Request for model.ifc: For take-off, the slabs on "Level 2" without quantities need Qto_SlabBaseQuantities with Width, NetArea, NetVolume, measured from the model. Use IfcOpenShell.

First a look at what the model holds.

```python
import ifcopenshell
import ifcopenshell.util.element
import ifcopenshell.util.unit

model = ifcopenshell.open("model.ifc")
print(model.schema)
for unit_type in ("LENGTHUNIT", "AREAUNIT", "VOLUMEUNIT"):
    print(unit_type, ifcopenshell.util.unit.calculate_unit_scale(model, unit_type))
storey = next(s for s in model.by_type("IfcBuildingStorey") if s.Name == "Level 2")
slabs = [e for e in ifcopenshell.util.element.get_decomposition(storey) if e.is_a("IfcSlab")]
for e in sorted(slabs, key=lambda e: e.id()):
    print(e.id(), e.is_a(), e.Name, list(ifcopenshell.util.element.get_psets(e, qtos_only=True)), sep=" | ")
```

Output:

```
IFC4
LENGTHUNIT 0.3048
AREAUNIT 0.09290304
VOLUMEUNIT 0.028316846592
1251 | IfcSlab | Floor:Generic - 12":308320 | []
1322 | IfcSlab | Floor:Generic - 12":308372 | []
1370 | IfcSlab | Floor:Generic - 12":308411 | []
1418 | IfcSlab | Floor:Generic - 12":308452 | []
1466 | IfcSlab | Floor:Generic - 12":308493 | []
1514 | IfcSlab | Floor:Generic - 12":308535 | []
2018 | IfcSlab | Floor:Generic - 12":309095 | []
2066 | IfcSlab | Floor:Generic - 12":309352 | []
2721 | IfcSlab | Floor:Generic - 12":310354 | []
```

```python
import ifcopenshell
import ifcopenshell.api.pset
import ifcopenshell.geom
import ifcopenshell.util.element
import ifcopenshell.util.shape
import ifcopenshell.util.unit

model = ifcopenshell.open("model.ifc")
unit_scale = ifcopenshell.util.unit.calculate_unit_scale(model)
area_scale = ifcopenshell.util.unit.calculate_unit_scale(model, "AREAUNIT")
volume_scale = ifcopenshell.util.unit.calculate_unit_scale(model, "VOLUMEUNIT")
settings = ifcopenshell.geom.settings()

storey = next(s for s in model.by_type("IfcBuildingStorey") if s.Name == "Level 2")
slabs = [e for e in ifcopenshell.util.element.get_decomposition(storey) if e.is_a("IfcSlab")]

for e in sorted(slabs, key=lambda e: e.id()):
    if ifcopenshell.util.element.get_psets(e, qtos_only=True, should_inherit=False):
        continue
    # Geometry comes back in metres, in the element's own axes.
    shape = ifcopenshell.geom.create_shape(settings, e)
    values = {
        "Width": ifcopenshell.util.shape.get_z(shape.geometry) / unit_scale,
        "NetArea": ifcopenshell.util.shape.get_footprint_area(shape.geometry) / area_scale,
        "NetVolume": ifcopenshell.util.shape.get_volume(shape.geometry) / volume_scale,
    }
    qto = ifcopenshell.api.pset.add_qto(model, product=e, name="Qto_SlabBaseQuantities")
    ifcopenshell.api.pset.edit_qto(model, qto=qto, properties=values)
    print(e.id(), {k: round(v, 3) for k, v in values.items()})

model.write("model_updated.ifc")
```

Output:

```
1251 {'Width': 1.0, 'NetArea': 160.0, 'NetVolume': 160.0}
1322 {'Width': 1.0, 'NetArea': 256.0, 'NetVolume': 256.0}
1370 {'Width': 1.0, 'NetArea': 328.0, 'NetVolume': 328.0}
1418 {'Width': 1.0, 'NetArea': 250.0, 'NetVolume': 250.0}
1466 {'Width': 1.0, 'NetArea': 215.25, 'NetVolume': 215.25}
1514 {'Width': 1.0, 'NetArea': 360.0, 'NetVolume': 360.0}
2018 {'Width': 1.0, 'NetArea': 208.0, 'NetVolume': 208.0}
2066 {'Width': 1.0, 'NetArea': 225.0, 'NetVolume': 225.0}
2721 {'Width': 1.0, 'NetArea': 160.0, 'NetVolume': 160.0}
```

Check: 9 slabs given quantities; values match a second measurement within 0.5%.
